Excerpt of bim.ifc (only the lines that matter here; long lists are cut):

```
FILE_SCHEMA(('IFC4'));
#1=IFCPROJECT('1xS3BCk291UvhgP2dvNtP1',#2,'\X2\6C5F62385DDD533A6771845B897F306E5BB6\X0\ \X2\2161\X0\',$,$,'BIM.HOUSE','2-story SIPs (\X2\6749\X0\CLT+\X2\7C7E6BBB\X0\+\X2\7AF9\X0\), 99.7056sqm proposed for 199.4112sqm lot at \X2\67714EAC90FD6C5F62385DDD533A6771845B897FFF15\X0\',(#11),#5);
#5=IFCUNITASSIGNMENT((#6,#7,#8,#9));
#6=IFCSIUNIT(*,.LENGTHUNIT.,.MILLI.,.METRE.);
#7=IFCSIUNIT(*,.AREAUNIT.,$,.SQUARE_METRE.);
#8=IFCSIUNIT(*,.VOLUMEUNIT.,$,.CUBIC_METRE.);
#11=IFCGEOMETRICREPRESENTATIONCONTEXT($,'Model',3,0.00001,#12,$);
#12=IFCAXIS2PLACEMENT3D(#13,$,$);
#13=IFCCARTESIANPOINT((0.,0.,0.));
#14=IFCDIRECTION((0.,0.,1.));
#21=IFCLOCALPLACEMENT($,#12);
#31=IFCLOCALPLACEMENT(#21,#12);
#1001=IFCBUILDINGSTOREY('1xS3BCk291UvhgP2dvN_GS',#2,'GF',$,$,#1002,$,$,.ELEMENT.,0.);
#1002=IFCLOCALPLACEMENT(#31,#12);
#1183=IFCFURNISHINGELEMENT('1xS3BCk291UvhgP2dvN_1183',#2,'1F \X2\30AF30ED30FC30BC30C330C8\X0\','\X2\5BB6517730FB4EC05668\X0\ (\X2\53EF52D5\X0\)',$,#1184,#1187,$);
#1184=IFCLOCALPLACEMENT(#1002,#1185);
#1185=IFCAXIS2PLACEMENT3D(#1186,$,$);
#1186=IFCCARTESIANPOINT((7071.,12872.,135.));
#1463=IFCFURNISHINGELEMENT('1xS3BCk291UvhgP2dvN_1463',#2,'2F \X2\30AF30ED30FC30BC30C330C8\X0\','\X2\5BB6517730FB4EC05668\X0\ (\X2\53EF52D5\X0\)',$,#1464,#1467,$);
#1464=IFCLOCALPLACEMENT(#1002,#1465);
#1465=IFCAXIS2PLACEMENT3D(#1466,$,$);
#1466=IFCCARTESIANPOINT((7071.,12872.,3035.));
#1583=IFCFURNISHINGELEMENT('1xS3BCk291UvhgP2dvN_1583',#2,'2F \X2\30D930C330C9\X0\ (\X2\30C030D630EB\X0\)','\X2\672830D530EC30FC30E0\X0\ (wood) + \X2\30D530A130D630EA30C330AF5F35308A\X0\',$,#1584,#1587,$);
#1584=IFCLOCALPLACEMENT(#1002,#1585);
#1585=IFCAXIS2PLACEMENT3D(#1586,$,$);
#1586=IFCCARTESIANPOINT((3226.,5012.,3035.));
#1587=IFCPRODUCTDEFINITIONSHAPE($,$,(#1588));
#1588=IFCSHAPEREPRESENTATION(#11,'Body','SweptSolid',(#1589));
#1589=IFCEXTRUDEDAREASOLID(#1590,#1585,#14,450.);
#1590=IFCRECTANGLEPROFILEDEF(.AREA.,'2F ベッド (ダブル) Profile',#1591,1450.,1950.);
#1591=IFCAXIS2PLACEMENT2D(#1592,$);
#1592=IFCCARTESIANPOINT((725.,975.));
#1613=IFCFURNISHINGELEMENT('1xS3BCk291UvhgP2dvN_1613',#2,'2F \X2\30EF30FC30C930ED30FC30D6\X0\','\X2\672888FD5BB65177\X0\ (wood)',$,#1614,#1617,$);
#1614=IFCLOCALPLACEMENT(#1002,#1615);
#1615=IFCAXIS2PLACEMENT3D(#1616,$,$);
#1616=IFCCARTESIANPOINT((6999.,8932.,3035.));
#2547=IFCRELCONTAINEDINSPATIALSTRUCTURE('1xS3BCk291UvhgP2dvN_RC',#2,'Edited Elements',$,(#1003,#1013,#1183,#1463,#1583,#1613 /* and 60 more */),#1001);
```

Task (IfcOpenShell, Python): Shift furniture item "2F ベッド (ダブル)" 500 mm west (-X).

```python
import ifcopenshell
import ifcopenshell.api.geometry
import ifcopenshell.util.placement

model = ifcopenshell.open("bim.ifc")

item = model.by_guid("1xS3BCk291UvhgP2dvN_1583")
matrix = ifcopenshell.util.placement.get_local_placement(item.ObjectPlacement)
matrix[0, 3] -= 500.0
ifcopenshell.api.geometry.edit_object_placement(model, product=item, matrix=matrix, is_si=False)

print(ifcopenshell.util.placement.get_local_placement(item.ObjectPlacement).round(3) + 0.0)

model.write("bim_updated.ifc")
```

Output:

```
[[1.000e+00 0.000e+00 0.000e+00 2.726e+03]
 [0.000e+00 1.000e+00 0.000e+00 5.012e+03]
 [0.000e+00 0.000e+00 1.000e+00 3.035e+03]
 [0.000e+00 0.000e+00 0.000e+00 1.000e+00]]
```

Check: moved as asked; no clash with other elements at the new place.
